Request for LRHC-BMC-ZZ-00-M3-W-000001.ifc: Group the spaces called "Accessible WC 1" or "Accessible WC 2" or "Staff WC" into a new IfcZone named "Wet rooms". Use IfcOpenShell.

First a look at what the model holds.

```python
import ifcopenshell

model = ifcopenshell.open("LRHC-BMC-ZZ-00-M3-W-000001.ifc")
print(model.schema)
seen = {}
for space in model.by_type("IfcSpace"):
    seen[space.LongName] = seen.get(space.LongName, 0) + 1
for name, count in sorted(seen.items(), key=str):
    print(count, "x", name)
print("zones:", [z.Name for z in model.by_type("IfcZone")][:20])
```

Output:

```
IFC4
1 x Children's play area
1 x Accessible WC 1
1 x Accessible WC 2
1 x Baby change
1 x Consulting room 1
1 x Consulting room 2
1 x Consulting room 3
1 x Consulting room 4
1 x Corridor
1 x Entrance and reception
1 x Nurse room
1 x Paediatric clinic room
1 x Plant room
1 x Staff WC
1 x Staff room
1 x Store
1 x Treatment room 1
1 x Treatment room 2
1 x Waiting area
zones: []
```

```python
import ifcopenshell
import ifcopenshell.api.group
import ifcopenshell.api.root

model = ifcopenshell.open("LRHC-BMC-ZZ-00-M3-W-000001.ifc")

names = {"Accessible WC 1", "Accessible WC 2", "Staff WC"}
spaces = [s for s in model.by_type("IfcSpace") if s.LongName in names]

zone = ifcopenshell.api.root.create_entity(model, ifc_class="IfcZone", name="Wet rooms")
ifcopenshell.api.group.assign_group(model, products=spaces, group=zone)
print(len(spaces), "spaces in", zone.Name)

model.write("LRHC-BMC-ZZ-00-M3-W-000001_v2.ifc")
```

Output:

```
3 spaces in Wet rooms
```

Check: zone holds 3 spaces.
